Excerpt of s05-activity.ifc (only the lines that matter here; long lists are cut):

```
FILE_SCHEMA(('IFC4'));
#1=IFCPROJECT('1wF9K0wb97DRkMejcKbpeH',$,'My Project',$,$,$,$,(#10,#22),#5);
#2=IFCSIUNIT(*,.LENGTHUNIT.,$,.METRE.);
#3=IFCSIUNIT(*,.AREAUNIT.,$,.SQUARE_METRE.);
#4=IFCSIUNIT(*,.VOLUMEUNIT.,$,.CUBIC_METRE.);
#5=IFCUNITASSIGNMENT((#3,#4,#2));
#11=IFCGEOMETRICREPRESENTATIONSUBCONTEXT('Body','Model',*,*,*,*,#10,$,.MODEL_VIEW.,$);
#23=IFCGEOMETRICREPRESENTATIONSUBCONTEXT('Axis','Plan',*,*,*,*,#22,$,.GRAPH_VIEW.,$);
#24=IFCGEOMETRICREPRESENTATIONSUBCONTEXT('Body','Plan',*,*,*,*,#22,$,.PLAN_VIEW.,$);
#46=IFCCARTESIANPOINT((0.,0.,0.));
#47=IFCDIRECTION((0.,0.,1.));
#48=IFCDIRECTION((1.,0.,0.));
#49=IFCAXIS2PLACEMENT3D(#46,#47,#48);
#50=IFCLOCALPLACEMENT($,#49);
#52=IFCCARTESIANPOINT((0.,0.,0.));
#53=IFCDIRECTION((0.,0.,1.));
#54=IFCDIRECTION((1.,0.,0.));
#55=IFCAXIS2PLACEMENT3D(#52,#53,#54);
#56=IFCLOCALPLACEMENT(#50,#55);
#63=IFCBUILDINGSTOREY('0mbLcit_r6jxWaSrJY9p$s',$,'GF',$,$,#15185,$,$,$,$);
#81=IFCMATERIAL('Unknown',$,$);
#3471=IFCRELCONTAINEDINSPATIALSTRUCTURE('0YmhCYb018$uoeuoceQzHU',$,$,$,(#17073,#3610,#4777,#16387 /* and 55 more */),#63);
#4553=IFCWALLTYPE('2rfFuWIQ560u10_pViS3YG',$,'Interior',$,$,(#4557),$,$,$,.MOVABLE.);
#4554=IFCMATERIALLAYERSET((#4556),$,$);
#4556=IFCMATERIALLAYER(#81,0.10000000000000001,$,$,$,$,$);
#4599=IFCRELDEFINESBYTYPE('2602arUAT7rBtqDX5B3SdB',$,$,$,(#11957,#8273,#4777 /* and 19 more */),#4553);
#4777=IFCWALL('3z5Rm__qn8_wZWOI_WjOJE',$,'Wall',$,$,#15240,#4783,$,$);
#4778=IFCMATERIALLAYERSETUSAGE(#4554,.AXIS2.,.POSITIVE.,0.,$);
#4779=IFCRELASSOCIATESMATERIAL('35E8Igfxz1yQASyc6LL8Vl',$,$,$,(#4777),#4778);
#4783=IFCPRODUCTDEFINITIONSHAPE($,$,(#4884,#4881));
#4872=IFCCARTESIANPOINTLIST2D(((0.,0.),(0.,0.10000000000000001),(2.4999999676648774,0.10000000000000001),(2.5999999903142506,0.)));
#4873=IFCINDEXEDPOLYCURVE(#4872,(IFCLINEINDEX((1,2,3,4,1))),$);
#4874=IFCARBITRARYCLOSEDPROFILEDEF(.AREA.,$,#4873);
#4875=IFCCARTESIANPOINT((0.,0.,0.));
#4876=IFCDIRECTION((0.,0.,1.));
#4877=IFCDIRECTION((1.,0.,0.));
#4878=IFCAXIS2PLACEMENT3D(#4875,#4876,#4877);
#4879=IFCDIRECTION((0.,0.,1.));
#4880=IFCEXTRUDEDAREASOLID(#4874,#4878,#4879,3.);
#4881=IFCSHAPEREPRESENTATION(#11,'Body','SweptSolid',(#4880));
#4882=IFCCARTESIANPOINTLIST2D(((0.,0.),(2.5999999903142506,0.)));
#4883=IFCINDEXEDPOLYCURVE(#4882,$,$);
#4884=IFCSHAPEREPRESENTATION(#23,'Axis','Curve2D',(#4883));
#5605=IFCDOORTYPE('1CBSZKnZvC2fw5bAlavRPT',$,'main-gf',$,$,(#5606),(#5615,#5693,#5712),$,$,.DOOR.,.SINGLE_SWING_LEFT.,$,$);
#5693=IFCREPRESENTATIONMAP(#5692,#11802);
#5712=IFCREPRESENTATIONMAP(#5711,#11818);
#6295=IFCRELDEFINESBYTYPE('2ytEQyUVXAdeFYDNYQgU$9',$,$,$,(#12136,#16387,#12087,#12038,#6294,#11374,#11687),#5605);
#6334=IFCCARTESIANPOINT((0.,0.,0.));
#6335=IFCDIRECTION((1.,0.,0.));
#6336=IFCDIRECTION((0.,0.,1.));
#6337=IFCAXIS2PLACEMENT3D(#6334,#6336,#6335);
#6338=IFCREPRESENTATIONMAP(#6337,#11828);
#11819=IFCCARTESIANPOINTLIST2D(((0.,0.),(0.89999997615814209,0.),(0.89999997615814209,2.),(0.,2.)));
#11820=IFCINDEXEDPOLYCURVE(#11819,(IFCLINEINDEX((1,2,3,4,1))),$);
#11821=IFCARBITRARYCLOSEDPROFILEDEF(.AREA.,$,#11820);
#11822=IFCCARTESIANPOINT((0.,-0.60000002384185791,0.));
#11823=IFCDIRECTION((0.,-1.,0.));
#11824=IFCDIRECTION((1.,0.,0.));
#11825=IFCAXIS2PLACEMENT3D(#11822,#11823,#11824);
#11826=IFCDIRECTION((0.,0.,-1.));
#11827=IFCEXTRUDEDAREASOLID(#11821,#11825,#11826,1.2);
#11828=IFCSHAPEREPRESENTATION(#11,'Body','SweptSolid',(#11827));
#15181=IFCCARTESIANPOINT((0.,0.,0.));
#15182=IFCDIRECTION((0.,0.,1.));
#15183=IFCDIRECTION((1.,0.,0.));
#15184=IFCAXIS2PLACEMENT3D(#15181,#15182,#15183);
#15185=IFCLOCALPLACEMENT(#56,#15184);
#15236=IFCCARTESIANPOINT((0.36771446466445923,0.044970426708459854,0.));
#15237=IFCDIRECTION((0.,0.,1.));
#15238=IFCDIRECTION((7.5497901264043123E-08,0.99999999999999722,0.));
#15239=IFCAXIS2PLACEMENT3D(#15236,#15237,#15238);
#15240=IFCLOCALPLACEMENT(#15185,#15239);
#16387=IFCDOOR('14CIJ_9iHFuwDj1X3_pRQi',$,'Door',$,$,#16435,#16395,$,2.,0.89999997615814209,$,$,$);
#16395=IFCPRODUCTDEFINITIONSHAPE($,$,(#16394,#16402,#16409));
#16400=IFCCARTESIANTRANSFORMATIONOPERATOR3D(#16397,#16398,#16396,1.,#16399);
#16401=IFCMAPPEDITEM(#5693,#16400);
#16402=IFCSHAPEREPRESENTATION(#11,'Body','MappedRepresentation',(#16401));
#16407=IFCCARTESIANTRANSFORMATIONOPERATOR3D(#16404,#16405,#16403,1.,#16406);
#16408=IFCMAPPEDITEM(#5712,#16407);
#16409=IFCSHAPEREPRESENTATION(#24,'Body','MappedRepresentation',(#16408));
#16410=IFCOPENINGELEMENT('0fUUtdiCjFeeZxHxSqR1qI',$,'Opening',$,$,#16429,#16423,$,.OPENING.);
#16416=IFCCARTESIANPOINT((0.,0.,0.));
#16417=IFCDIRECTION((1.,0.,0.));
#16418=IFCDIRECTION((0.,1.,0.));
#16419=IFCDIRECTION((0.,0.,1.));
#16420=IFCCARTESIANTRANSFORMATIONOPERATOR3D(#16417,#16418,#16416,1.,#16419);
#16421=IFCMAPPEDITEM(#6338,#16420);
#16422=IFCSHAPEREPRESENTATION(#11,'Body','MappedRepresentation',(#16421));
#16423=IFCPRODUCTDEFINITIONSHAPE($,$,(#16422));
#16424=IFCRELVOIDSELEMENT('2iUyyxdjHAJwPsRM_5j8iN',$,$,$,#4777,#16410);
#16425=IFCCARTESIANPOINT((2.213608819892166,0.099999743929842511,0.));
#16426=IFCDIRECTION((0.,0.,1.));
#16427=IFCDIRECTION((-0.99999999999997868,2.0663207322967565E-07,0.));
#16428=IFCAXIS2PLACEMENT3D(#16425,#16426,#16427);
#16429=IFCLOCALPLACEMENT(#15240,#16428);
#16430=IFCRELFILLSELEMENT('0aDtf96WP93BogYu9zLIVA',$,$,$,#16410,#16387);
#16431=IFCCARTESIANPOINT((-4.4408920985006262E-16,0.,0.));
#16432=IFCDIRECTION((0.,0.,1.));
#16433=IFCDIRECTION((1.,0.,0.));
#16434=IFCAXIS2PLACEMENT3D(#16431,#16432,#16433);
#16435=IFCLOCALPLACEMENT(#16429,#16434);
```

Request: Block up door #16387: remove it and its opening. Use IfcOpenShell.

```python
import ifcopenshell
import ifcopenshell.api.feature
import ifcopenshell.api.root
import ifcopenshell.geom
import ifcopenshell.util.shape

model = ifcopenshell.open("s05-activity.ifc")
settings = ifcopenshell.geom.settings()


def volume(element):
    """Net volume in cubic metres, openings subtracted."""
    shape = ifcopenshell.geom.create_shape(settings, element)
    return ifcopenshell.util.shape.get_volume(shape.geometry)


door = model.by_guid("14CIJ_9iHFuwDj1X3_pRQi")
opening = door.FillsVoids[0].RelatingOpeningElement
wall = opening.VoidsElements[0].RelatingBuildingElement
before = volume(wall)

ifcopenshell.api.root.remove_product(model, product=door)
ifcopenshell.api.feature.remove_feature(model, feature=opening)

after = volume(wall)

print(f"wall volume {before:.3f} -> {after:.3f} m3")

model.write("s05-activity_updated.ifc")
```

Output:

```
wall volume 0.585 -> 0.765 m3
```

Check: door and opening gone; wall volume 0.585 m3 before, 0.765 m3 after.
